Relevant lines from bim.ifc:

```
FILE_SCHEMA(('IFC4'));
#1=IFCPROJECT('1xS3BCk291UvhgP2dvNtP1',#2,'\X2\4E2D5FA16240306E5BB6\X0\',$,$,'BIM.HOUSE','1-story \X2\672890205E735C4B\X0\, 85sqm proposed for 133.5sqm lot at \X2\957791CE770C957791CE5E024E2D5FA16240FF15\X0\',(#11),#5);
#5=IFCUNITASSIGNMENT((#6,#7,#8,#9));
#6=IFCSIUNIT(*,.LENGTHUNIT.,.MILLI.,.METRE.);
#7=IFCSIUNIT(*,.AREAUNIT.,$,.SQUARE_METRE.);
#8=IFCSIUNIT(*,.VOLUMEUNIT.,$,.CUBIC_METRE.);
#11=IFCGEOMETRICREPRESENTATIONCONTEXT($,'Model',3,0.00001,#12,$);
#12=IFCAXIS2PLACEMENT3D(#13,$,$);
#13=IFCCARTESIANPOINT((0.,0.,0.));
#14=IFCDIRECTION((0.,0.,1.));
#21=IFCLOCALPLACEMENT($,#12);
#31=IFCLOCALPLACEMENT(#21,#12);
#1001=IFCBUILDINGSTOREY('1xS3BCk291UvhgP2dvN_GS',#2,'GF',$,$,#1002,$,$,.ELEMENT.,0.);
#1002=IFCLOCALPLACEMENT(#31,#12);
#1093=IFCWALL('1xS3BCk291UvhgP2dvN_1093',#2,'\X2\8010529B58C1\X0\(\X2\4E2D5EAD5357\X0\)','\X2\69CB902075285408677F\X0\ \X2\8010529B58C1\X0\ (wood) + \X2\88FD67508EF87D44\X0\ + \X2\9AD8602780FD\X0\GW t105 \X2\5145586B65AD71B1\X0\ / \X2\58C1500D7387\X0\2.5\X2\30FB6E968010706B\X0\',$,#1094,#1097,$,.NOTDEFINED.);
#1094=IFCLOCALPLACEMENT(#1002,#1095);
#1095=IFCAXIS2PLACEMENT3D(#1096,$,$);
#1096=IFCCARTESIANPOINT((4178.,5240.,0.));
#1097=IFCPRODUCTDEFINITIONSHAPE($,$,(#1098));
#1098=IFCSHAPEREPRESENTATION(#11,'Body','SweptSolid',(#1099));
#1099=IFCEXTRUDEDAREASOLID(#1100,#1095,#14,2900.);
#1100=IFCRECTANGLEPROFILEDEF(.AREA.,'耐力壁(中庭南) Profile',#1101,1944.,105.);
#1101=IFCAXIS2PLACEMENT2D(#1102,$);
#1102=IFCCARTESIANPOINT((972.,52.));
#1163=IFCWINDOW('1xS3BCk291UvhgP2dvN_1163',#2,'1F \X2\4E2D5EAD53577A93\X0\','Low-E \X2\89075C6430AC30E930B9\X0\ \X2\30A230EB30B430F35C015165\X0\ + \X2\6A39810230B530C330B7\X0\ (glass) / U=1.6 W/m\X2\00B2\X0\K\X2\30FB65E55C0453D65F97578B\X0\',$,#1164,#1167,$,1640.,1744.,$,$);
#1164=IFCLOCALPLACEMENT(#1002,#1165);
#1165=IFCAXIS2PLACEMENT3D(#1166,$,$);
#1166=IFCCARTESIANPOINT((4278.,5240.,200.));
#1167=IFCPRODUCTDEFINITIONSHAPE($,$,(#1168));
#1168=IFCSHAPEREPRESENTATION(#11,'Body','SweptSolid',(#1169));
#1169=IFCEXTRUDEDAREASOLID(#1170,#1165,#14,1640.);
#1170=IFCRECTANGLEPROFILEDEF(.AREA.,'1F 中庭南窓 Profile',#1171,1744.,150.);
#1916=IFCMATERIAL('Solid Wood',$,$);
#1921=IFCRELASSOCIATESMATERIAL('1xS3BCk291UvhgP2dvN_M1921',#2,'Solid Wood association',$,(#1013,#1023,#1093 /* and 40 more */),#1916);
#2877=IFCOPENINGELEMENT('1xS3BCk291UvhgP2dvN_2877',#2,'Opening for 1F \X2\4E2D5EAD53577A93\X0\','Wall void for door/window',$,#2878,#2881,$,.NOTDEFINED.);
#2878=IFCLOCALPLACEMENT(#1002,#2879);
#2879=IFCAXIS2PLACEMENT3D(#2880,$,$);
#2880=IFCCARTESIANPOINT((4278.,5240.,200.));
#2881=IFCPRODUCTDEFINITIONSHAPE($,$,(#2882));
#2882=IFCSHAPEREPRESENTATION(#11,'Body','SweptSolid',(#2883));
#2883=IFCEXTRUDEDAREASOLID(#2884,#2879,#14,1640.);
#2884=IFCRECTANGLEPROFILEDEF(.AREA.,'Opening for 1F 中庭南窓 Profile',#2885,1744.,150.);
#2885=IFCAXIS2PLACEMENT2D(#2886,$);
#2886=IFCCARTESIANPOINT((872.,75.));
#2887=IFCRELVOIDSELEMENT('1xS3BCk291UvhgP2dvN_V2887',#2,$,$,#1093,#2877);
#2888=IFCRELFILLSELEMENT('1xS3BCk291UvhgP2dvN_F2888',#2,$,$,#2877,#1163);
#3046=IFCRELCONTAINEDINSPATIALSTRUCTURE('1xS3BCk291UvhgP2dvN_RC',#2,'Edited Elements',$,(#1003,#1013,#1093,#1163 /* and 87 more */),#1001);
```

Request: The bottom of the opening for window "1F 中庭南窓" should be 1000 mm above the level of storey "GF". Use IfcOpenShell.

```python
import numpy as np
import ifcopenshell
import ifcopenshell.api.geometry
import ifcopenshell.geom
import ifcopenshell.util.element
import ifcopenshell.util.placement
import ifcopenshell.util.shape
import ifcopenshell.util.unit

model = ifcopenshell.open("bim.ifc")
unit_scale = ifcopenshell.util.unit.calculate_unit_scale(model)

window = model.by_id(1163)
opening = window.FillsVoids[0].RelatingOpeningElement
storey = ifcopenshell.util.element.get_container(window, ifc_class="IfcBuildingStorey")
level = ifcopenshell.util.placement.get_local_placement(storey.ObjectPlacement)[2, 3]

# The opening's origin need not be at the sill, so measure its lowest point.
shape = ifcopenshell.geom.create_shape(ifcopenshell.geom.settings(), opening)
bottom = ifcopenshell.util.shape.get_shape_bottom_elevation(shape, shape.geometry) / unit_scale
dz = level + 1 / unit_scale - bottom

shift = np.array([0.0, 0.0, dz])
# The window is not placed relative to its opening, so move both.
for product in (opening, window):
    matrix = ifcopenshell.util.placement.get_local_placement(product.ObjectPlacement)
    matrix[:3, 3] += shift
    ifcopenshell.api.geometry.edit_object_placement(model, product=product, matrix=matrix, is_si=False)

print(f"moved by {dz * unit_scale:+.3f} m")

model.write("bim_rev.ifc")
```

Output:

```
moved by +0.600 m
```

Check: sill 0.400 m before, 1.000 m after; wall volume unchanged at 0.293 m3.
